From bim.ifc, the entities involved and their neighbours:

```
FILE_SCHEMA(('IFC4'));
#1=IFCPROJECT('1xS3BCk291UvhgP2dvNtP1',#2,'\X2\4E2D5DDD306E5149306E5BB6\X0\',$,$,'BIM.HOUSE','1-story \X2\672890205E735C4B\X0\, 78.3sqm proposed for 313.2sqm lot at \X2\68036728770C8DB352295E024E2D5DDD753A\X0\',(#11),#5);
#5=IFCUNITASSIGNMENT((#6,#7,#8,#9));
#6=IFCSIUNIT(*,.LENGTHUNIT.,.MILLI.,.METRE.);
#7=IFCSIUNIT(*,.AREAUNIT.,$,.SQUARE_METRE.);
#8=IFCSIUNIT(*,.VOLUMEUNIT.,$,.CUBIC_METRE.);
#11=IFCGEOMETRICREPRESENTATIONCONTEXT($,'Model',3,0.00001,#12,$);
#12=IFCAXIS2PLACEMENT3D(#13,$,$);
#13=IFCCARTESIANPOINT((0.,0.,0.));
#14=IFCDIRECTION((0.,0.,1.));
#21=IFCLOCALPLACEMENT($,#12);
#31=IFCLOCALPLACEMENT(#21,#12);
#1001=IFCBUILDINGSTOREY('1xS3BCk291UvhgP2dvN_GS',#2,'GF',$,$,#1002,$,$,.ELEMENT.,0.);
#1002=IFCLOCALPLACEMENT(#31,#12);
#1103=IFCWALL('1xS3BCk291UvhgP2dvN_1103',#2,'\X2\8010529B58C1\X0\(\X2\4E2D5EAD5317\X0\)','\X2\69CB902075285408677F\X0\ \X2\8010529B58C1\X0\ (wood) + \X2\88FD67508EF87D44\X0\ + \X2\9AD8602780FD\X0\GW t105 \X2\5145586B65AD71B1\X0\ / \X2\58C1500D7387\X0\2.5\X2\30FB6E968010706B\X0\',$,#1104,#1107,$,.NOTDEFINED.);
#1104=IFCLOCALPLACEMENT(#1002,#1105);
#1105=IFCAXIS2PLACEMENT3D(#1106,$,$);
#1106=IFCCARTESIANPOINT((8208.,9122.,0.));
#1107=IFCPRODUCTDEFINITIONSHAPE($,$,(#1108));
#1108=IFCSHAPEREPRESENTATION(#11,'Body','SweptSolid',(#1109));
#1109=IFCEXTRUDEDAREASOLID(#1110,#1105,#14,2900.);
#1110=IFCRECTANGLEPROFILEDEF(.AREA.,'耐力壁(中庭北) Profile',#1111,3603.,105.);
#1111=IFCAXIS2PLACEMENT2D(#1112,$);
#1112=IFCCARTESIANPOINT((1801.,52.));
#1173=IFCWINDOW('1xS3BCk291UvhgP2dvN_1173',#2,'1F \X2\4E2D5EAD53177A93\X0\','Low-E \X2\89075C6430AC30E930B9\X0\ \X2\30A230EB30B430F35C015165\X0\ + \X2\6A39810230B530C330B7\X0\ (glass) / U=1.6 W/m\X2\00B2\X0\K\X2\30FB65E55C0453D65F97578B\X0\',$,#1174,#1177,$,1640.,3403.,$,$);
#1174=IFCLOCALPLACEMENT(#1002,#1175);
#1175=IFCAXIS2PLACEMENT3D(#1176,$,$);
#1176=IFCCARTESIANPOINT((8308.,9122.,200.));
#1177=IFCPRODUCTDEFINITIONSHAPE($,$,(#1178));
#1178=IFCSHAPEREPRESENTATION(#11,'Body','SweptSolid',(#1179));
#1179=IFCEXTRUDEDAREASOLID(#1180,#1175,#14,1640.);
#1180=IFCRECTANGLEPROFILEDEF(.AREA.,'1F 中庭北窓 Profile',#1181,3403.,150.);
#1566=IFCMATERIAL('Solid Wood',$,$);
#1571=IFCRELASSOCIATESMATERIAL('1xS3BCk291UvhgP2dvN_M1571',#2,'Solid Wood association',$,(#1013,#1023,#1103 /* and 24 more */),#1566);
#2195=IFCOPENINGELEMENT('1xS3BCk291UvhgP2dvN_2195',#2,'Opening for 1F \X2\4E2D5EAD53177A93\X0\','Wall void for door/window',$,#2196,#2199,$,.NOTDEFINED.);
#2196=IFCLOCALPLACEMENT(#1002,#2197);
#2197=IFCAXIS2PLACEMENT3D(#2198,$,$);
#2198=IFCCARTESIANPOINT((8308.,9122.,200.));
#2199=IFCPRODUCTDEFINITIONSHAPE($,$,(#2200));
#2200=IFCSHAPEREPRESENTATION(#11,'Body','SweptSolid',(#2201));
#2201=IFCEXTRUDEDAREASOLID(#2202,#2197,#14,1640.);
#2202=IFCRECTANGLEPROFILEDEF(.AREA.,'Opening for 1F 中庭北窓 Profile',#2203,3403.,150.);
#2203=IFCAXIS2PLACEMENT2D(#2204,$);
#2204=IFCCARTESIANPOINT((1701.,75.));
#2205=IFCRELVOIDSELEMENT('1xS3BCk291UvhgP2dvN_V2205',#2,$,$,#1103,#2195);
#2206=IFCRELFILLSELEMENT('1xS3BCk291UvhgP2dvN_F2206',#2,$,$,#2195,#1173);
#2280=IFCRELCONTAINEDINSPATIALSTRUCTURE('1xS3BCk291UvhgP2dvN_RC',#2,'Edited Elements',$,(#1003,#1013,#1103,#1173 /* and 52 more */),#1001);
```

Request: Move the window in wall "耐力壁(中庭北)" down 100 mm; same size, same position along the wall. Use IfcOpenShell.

```python
import numpy as np
import ifcopenshell
import ifcopenshell.api.geometry
import ifcopenshell.util.placement
import ifcopenshell.util.unit

model = ifcopenshell.open("bim.ifc")
unit_scale = ifcopenshell.util.unit.calculate_unit_scale(model)

window = model.by_guid("1xS3BCk291UvhgP2dvN_1173")
opening = window.FillsVoids[0].RelatingOpeningElement
dz = -0.1 / unit_scale

shift = np.array([0.0, 0.0, dz])
# The window is not placed relative to its opening, so move both.
for product in (opening, window):
    matrix = ifcopenshell.util.placement.get_local_placement(product.ObjectPlacement)
    matrix[:3, 3] += shift
    ifcopenshell.api.geometry.edit_object_placement(model, product=product, matrix=matrix, is_si=False)

print(f"moved by {dz * unit_scale:+.3f} m")

model.write("bim_edited.ifc")
```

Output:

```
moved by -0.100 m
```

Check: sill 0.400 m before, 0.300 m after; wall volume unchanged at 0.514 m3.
